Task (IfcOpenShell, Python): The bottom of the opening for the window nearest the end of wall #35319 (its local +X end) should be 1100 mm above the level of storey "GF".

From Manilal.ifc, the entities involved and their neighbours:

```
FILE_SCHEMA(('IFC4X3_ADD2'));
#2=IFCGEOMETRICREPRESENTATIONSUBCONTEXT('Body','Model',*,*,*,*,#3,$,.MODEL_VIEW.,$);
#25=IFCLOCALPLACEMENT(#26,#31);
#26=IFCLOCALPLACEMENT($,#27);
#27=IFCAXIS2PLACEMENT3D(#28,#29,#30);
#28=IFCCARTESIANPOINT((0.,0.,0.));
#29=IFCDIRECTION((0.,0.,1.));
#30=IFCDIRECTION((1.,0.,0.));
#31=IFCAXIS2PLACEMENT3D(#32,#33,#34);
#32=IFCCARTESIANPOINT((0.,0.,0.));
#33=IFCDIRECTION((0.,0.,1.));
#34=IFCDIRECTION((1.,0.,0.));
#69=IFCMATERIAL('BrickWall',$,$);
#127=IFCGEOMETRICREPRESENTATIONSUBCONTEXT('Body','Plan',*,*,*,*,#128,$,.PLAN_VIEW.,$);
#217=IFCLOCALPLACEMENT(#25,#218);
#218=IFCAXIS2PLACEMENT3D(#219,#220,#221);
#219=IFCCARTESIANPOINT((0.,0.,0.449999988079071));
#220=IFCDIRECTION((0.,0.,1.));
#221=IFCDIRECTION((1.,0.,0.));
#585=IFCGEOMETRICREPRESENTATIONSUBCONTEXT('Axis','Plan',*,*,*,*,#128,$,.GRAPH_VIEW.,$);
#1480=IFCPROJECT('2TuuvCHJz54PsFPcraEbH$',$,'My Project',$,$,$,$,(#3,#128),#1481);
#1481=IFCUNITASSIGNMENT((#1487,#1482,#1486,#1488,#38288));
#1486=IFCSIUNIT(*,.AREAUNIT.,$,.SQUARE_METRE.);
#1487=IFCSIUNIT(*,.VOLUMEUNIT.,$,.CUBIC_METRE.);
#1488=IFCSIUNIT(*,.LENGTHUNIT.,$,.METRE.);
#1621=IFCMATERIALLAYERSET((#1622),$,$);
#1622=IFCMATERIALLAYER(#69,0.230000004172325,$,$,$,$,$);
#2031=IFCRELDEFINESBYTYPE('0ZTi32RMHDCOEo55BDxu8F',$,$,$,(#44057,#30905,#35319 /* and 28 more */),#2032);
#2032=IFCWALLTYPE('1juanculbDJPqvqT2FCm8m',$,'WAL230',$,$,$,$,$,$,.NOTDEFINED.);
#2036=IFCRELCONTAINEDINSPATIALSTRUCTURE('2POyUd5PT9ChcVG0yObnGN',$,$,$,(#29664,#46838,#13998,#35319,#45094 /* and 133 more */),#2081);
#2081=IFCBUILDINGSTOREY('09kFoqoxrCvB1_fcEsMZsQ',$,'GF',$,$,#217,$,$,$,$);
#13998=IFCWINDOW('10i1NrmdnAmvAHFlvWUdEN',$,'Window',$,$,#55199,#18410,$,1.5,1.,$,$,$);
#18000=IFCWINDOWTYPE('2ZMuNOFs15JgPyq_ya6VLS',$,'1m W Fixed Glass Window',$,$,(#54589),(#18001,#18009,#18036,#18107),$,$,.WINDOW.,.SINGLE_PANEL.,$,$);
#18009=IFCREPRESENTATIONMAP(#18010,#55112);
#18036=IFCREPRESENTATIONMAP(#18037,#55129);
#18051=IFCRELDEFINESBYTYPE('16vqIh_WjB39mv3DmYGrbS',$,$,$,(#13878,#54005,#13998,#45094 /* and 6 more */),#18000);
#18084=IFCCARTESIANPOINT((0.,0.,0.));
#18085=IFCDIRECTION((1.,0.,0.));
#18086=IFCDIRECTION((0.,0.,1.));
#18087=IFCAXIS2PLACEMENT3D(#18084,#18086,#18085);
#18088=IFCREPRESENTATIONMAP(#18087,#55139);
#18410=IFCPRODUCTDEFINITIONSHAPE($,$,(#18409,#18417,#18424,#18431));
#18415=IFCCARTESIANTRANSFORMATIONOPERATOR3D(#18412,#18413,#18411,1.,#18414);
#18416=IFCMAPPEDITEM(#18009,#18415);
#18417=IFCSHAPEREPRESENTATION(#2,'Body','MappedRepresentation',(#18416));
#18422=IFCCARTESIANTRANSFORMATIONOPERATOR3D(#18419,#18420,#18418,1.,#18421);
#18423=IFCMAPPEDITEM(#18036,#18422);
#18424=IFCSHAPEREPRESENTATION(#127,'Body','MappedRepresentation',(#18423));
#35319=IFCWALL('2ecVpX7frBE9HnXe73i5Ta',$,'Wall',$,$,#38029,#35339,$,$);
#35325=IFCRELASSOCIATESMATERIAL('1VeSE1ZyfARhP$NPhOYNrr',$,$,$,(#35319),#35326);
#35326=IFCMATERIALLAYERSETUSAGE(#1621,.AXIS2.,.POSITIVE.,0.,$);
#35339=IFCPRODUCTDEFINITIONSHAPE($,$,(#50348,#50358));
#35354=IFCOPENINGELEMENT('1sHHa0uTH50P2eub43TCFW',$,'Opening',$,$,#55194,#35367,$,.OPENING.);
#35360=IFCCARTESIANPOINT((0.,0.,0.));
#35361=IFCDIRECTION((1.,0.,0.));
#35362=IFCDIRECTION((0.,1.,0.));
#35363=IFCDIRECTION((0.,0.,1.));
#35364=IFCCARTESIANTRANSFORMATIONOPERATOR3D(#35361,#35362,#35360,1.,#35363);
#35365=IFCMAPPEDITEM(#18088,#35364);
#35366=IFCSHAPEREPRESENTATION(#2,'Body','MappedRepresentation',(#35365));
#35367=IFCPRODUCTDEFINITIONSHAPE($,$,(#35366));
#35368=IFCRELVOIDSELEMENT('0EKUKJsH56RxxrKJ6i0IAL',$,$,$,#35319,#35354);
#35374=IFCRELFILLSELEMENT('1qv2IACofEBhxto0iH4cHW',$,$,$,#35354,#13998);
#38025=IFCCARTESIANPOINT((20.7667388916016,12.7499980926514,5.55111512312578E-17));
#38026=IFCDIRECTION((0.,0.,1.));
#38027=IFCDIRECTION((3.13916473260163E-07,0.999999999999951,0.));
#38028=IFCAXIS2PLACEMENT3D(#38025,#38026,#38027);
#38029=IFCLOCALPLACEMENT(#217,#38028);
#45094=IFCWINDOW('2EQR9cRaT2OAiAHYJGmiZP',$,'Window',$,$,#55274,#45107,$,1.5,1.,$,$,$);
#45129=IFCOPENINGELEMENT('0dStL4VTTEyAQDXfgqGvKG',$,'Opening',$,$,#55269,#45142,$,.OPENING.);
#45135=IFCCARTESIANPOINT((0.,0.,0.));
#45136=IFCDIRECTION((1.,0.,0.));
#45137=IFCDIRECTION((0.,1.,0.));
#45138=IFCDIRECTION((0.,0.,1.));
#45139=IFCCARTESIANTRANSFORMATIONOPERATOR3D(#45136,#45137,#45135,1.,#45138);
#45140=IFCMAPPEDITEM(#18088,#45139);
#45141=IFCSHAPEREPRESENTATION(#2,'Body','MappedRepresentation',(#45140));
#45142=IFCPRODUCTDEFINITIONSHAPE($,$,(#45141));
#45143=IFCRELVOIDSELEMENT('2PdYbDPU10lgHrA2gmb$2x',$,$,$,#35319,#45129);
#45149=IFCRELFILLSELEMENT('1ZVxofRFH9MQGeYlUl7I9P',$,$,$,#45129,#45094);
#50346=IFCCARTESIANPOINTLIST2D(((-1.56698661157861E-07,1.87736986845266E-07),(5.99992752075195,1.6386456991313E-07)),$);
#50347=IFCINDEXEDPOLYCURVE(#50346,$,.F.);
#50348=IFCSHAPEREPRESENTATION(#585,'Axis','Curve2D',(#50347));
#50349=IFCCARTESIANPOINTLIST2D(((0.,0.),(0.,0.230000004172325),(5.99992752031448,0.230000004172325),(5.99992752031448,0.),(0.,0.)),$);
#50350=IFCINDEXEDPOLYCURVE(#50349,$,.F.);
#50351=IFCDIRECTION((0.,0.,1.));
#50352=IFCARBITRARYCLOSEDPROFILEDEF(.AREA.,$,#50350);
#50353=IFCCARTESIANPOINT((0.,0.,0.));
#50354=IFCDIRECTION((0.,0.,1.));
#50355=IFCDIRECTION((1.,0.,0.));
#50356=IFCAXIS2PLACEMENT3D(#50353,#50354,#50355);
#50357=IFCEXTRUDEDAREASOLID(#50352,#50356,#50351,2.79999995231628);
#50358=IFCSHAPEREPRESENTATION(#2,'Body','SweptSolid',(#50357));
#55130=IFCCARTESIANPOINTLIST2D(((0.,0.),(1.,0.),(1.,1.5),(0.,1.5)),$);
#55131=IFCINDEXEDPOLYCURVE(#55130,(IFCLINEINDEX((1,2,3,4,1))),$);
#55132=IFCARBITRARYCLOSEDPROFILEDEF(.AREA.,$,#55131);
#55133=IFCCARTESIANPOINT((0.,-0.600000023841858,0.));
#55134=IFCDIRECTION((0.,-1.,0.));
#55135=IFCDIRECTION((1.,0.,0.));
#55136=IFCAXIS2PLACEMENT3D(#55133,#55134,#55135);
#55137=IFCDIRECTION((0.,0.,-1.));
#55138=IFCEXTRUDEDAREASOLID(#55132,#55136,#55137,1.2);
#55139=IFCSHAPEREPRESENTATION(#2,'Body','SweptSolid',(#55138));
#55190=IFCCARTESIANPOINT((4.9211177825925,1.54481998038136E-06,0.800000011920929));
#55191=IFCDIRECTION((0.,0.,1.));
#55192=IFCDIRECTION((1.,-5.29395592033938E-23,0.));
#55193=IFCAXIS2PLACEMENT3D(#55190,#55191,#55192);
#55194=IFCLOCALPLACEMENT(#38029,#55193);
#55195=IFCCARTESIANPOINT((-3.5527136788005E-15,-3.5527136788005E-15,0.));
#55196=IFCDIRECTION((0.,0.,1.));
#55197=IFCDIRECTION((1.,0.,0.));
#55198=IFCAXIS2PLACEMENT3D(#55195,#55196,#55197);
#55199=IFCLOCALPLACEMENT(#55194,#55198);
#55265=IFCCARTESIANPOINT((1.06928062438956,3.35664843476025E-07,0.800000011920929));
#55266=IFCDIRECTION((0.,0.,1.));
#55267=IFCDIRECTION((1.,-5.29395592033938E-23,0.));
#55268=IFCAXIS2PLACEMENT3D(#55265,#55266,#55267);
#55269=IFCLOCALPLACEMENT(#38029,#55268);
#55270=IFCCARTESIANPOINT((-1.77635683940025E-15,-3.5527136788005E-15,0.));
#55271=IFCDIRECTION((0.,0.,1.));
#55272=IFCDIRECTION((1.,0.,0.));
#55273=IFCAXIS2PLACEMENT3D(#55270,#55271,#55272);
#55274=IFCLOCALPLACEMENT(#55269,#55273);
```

```python
import numpy as np
import ifcopenshell
import ifcopenshell.api.geometry
import ifcopenshell.geom
import ifcopenshell.util.element
import ifcopenshell.util.placement
import ifcopenshell.util.shape
import ifcopenshell.util.unit

model = ifcopenshell.open("Manilal.ifc")
unit_scale = ifcopenshell.util.unit.calculate_unit_scale(model)

window = model.by_guid("10i1NrmdnAmvAHFlvWUdEN")
opening = window.FillsVoids[0].RelatingOpeningElement
storey = ifcopenshell.util.element.get_container(window, ifc_class="IfcBuildingStorey")
level = ifcopenshell.util.placement.get_local_placement(storey.ObjectPlacement)[2, 3]

# The opening's origin need not be at the sill, so measure its lowest point.
shape = ifcopenshell.geom.create_shape(ifcopenshell.geom.settings(), opening)
bottom = ifcopenshell.util.shape.get_shape_bottom_elevation(shape, shape.geometry) / unit_scale
dz = level + 1.1 / unit_scale - bottom

shift = np.array([0.0, 0.0, dz])
# The window is placed relative to its opening, so it follows when the opening moves.
matrix = ifcopenshell.util.placement.get_local_placement(opening.ObjectPlacement)
matrix[:3, 3] += shift
ifcopenshell.api.geometry.edit_object_placement(
    model, product=opening, matrix=matrix, is_si=False, should_transform_children=True
)

print(f"moved by {dz * unit_scale:+.3f} m")

model.write("Manilal_updated.ifc")
```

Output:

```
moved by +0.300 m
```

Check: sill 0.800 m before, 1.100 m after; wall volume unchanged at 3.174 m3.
